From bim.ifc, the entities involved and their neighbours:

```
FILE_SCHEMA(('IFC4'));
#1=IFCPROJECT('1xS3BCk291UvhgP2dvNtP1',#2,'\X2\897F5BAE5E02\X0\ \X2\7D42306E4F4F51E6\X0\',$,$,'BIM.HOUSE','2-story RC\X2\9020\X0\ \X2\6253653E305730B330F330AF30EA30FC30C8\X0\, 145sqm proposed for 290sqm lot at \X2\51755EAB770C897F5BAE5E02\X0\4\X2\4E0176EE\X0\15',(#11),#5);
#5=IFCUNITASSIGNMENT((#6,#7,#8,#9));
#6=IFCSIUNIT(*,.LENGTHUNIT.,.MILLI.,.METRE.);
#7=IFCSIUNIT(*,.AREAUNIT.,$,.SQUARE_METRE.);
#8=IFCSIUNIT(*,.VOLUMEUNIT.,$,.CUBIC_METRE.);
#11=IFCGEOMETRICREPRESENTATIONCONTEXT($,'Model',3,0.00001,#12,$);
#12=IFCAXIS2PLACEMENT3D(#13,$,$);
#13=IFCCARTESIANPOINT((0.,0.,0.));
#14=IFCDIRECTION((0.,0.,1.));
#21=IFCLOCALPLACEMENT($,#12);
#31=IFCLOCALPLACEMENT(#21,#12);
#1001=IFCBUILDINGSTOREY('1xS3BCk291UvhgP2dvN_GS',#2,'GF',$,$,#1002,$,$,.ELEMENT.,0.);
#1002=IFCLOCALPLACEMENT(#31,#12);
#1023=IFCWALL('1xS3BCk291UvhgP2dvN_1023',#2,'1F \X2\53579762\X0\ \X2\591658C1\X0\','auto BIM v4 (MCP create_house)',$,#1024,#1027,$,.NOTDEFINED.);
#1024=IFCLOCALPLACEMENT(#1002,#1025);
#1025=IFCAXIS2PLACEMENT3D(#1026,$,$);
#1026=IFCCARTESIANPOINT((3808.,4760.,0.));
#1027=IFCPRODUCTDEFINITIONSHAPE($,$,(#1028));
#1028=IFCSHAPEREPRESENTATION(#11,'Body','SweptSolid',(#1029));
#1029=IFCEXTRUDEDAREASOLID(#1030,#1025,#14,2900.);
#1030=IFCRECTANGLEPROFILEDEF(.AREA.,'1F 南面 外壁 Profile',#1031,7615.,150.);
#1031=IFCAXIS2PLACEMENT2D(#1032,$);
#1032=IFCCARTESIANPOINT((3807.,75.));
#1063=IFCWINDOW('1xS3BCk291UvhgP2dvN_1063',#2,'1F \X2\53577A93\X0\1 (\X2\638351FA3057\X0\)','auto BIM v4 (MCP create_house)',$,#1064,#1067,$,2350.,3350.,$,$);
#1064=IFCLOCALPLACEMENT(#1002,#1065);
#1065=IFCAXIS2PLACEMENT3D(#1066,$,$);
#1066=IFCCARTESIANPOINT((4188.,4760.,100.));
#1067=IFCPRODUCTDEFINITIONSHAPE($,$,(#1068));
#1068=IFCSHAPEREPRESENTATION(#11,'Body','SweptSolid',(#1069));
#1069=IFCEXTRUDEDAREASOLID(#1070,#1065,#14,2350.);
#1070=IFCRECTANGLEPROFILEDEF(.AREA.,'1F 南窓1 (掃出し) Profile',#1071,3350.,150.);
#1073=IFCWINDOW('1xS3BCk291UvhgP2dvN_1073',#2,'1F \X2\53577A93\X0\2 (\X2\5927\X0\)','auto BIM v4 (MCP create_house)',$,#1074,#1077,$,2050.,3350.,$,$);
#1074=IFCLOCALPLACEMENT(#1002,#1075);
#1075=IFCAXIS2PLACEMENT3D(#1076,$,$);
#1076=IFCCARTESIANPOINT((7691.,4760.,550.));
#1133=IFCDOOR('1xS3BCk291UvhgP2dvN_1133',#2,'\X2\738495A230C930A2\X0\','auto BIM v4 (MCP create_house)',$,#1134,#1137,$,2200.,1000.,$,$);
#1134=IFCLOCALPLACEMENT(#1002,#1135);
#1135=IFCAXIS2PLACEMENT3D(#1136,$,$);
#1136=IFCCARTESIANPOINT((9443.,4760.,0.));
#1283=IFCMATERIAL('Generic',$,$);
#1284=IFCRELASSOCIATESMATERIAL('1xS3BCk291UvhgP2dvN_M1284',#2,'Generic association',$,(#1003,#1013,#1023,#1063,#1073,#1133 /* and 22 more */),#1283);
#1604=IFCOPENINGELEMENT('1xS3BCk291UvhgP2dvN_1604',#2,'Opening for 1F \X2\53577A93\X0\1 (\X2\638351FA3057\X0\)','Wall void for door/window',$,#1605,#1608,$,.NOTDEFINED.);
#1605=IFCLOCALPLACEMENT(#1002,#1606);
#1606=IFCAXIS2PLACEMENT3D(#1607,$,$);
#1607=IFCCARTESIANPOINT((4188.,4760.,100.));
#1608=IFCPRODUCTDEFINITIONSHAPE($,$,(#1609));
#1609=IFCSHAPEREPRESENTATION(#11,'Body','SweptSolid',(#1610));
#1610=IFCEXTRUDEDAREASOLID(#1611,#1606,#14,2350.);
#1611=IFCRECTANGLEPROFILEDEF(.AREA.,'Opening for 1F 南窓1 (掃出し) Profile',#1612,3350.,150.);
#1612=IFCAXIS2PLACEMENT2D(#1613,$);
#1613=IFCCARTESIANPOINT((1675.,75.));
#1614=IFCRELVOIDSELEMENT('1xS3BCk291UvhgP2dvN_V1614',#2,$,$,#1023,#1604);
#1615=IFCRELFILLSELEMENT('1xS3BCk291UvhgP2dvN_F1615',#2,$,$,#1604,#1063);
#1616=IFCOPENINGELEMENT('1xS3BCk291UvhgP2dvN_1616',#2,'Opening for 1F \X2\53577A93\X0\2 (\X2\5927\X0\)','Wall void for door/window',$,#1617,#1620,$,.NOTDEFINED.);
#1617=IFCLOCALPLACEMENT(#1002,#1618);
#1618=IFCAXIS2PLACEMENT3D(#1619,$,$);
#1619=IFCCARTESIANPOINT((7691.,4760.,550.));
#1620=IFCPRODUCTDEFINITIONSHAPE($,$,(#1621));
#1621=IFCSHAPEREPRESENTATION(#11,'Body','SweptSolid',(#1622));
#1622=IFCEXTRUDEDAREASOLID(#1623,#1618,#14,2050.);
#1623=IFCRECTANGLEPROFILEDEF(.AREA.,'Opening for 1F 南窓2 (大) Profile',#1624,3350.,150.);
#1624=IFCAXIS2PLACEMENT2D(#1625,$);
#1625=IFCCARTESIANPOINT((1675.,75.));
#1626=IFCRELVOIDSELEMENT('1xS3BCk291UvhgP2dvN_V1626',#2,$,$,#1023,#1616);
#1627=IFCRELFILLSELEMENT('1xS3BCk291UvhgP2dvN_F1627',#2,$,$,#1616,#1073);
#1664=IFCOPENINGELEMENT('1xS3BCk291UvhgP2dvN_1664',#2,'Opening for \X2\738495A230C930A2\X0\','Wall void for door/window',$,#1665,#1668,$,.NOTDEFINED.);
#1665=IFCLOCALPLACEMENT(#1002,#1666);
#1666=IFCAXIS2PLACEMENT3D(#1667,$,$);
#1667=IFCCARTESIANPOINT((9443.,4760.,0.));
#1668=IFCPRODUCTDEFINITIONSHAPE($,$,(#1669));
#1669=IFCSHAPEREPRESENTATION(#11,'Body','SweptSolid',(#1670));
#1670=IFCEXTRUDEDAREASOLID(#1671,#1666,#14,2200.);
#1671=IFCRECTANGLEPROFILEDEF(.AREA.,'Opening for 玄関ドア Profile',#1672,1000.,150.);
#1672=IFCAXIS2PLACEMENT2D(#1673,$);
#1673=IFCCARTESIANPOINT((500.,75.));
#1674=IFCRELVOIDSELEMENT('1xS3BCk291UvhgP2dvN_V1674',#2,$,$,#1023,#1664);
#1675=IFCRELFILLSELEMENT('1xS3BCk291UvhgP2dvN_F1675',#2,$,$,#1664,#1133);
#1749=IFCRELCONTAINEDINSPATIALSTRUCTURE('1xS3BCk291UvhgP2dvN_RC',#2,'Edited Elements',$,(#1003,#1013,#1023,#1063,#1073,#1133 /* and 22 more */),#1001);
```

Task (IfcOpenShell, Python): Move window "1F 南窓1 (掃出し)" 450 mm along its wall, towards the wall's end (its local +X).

```python
import ifcopenshell
import ifcopenshell.api.geometry
import ifcopenshell.util.placement

model = ifcopenshell.open("bim.ifc")

window = model.by_id(1063)
opening = window.FillsVoids[0].RelatingOpeningElement
wall = opening.VoidsElements[0].RelatingBuildingElement

wall_matrix = ifcopenshell.util.placement.get_local_placement(wall.ObjectPlacement)
shift = wall_matrix[:3, 0] * 450.0
before = ifcopenshell.util.placement.get_local_placement(window.ObjectPlacement)[:3, 3].copy()

# The window is not placed relative to its opening, so move both.
for product in (opening, window):
    matrix = ifcopenshell.util.placement.get_local_placement(product.ObjectPlacement)
    matrix[:3, 3] += shift
    ifcopenshell.api.geometry.edit_object_placement(model, product=product, matrix=matrix, is_si=False)

after = ifcopenshell.util.placement.get_local_placement(window.ObjectPlacement)[:3, 3]
print("window moved by", (after - before).round(3) + 0.0)

model.write("bim_updated.ifc")
```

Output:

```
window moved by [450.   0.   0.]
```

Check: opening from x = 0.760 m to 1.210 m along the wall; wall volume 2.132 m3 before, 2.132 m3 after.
